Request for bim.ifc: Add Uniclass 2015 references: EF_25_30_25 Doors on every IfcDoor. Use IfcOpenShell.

First a look at what the model holds.

```python
import ifcopenshell

model = ifcopenshell.open("bim.ifc")
print(model.schema)
print("classifications:", [c.Name for c in model.by_type("IfcClassification")])
for ifc_class in ("IfcDoor", "IfcRoof", "IfcStair", "IfcWall", "IfcWindow"):
    print(ifc_class, len(model.by_type(ifc_class)))
```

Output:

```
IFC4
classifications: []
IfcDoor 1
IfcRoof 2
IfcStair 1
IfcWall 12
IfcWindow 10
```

```python
import ifcopenshell
import ifcopenshell.api.classification

model = ifcopenshell.open("bim.ifc")

system = ifcopenshell.api.classification.add_classification(model, classification="Uniclass 2015")

codes = {
    "IfcDoor": ("EF_25_30_25", "Doors"),
}
for ifc_class, (code, name) in codes.items():
    products = model.by_type(ifc_class)
    ifcopenshell.api.classification.add_reference(
        model, products=products, classification=system, identification=code, name=name
    )
    print(code, len(products))

model.write("bim_updated.ifc")
```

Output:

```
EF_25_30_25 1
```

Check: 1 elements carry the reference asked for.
